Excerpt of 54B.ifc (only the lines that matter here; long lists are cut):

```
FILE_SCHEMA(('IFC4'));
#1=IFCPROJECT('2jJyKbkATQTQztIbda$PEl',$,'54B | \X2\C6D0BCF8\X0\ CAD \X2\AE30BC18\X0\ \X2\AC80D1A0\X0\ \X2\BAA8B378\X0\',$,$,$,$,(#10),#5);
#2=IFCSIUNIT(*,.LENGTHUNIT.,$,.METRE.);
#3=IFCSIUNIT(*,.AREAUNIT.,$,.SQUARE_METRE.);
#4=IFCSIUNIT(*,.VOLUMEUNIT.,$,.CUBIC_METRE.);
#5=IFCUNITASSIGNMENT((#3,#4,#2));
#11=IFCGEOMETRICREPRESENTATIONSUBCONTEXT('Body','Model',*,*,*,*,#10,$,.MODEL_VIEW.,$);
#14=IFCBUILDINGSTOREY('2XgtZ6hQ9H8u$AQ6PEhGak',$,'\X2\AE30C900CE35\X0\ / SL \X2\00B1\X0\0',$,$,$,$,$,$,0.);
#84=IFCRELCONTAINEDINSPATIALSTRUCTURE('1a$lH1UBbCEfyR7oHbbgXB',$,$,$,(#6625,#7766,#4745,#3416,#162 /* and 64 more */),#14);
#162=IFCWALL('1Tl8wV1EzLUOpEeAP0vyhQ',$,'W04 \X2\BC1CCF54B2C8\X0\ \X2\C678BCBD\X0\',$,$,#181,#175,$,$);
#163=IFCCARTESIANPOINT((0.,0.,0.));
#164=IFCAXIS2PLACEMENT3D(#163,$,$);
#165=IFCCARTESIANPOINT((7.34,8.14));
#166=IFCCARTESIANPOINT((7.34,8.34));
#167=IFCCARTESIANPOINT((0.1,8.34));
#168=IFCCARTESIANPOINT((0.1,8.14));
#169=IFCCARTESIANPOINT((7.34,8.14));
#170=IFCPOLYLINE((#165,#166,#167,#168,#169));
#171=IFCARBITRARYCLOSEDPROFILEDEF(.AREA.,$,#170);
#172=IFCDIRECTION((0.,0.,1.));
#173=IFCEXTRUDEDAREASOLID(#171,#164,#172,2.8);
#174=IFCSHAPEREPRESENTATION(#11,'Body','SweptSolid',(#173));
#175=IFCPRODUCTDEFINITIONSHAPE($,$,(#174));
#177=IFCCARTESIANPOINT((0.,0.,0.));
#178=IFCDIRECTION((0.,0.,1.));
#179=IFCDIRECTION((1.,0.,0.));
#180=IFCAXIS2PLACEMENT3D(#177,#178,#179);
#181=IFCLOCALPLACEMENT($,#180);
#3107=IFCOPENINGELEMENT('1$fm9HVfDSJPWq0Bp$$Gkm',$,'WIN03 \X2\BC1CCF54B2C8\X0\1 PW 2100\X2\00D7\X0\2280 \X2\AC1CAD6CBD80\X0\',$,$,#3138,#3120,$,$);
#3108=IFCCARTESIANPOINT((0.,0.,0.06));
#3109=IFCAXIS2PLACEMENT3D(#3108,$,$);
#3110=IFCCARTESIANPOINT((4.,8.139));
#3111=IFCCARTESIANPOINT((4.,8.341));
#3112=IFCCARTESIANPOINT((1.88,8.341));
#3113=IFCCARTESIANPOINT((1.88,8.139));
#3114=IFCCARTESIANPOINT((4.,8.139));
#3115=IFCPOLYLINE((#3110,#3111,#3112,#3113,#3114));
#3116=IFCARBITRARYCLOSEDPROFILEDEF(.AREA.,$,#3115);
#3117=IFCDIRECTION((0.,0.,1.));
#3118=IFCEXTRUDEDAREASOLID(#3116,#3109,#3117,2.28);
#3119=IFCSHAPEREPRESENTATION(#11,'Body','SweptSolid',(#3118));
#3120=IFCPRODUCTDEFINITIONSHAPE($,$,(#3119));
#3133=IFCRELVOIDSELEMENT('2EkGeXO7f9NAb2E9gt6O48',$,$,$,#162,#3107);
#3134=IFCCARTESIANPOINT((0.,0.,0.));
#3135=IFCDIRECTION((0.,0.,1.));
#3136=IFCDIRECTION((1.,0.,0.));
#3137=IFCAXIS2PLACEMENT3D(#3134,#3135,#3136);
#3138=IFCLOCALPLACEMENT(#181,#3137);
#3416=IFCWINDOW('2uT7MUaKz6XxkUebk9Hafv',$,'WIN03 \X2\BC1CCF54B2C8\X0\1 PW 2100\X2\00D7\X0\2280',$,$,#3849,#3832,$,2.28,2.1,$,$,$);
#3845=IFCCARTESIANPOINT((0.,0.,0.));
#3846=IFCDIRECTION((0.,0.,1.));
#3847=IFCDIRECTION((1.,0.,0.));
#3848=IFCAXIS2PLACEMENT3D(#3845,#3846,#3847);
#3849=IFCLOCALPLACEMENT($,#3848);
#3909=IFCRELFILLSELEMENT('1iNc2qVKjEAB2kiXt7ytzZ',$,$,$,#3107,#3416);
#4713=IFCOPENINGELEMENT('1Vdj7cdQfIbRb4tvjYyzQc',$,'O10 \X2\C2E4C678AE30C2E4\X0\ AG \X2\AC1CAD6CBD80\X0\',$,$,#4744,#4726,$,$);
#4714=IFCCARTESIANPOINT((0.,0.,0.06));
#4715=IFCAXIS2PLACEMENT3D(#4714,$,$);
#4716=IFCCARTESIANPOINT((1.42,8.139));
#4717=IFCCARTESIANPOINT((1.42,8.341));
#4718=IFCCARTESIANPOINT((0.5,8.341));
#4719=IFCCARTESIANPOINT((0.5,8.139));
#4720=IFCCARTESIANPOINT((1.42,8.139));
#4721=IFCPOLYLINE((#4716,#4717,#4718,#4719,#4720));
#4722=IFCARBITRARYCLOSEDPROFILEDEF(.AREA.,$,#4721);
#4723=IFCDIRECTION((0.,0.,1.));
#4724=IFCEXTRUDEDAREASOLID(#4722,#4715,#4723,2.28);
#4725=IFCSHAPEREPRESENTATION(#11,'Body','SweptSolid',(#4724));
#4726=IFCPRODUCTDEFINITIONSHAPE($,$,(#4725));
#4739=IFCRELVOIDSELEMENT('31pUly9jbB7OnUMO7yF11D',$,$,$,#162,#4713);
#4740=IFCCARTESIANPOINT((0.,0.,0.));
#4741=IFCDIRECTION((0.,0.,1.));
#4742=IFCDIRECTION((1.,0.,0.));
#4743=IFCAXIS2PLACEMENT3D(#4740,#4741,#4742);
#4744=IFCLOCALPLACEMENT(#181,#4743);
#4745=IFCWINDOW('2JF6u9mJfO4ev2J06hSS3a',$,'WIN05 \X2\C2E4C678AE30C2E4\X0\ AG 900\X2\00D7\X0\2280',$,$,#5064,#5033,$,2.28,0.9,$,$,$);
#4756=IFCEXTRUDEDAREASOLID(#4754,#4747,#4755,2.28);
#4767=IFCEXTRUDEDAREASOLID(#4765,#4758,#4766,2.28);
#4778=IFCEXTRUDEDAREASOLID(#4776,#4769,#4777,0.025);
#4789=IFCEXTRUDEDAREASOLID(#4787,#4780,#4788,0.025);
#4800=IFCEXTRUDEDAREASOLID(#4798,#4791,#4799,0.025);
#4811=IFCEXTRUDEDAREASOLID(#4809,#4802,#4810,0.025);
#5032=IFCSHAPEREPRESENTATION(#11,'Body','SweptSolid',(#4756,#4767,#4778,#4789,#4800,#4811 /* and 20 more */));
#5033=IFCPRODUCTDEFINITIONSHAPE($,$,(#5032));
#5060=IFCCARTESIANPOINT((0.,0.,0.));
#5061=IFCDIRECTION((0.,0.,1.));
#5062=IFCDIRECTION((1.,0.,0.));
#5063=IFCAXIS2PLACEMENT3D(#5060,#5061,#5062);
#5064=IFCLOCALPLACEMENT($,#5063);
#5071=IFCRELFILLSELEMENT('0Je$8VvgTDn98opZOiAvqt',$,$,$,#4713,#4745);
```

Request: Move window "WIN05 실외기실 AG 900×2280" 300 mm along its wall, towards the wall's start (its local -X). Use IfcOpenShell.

```python
import ifcopenshell
import ifcopenshell.api.geometry
import ifcopenshell.util.placement

model = ifcopenshell.open("54B.ifc")

window = model.by_guid("2JF6u9mJfO4ev2J06hSS3a")
opening = window.FillsVoids[0].RelatingOpeningElement
wall = opening.VoidsElements[0].RelatingBuildingElement

wall_matrix = ifcopenshell.util.placement.get_local_placement(wall.ObjectPlacement)
shift = wall_matrix[:3, 0] * -0.3
before = ifcopenshell.util.placement.get_local_placement(window.ObjectPlacement)[:3, 3].copy()

# The window is not placed relative to its opening, so move both.
for product in (opening, window):
    matrix = ifcopenshell.util.placement.get_local_placement(product.ObjectPlacement)
    matrix[:3, 3] += shift
    ifcopenshell.api.geometry.edit_object_placement(model, product=product, matrix=matrix, is_si=False)

after = ifcopenshell.util.placement.get_local_placement(window.ObjectPlacement)[:3, 3]
print("window moved by", (after - before).round(3) + 0.0)

model.write("54B_v2.ifc")
```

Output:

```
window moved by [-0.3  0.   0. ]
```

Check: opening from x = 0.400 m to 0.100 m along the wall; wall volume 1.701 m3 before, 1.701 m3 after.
